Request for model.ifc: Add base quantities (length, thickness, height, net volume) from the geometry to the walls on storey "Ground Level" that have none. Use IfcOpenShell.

First a look at what the model holds.

```python
import ifcopenshell
import ifcopenshell.util.element
import ifcopenshell.util.unit

model = ifcopenshell.open("model.ifc")
print(model.schema)
for unit_type in ("LENGTHUNIT", "AREAUNIT", "VOLUMEUNIT"):
    print(unit_type, ifcopenshell.util.unit.calculate_unit_scale(model, unit_type))
storey = next(s for s in model.by_type("IfcBuildingStorey") if s.Name == "Ground Level")
walls = [e for e in ifcopenshell.util.element.get_decomposition(storey) if e.is_a("IfcWall")]
for e in sorted(walls, key=lambda e: e.id()):
    print(e.id(), e.is_a(), e.Name, list(ifcopenshell.util.element.get_psets(e, qtos_only=True)), sep=" | ")
```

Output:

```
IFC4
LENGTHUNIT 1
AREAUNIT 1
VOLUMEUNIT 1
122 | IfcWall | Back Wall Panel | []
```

```python
import ifcopenshell
import ifcopenshell.api.pset
import ifcopenshell.geom
import ifcopenshell.util.element
import ifcopenshell.util.shape
import ifcopenshell.util.unit

model = ifcopenshell.open("model.ifc")
unit_scale = ifcopenshell.util.unit.calculate_unit_scale(model)
volume_scale = ifcopenshell.util.unit.calculate_unit_scale(model, "VOLUMEUNIT")
settings = ifcopenshell.geom.settings()

storey = next(s for s in model.by_type("IfcBuildingStorey") if s.Name == "Ground Level")
walls = [e for e in ifcopenshell.util.element.get_decomposition(storey) if e.is_a("IfcWall")]

for e in sorted(walls, key=lambda e: e.id()):
    if ifcopenshell.util.element.get_psets(e, qtos_only=True, should_inherit=False):
        continue
    # Geometry comes back in metres, in the element's own axes.
    shape = ifcopenshell.geom.create_shape(settings, e)
    values = {
        "Length": ifcopenshell.util.shape.get_x(shape.geometry) / unit_scale,
        "Width": ifcopenshell.util.shape.get_y(shape.geometry) / unit_scale,
        "Height": ifcopenshell.util.shape.get_z(shape.geometry) / unit_scale,
        "NetVolume": ifcopenshell.util.shape.get_volume(shape.geometry) / volume_scale,
    }
    qto = ifcopenshell.api.pset.add_qto(model, product=e, name="Qto_WallBaseQuantities")
    ifcopenshell.api.pset.edit_qto(model, qto=qto, properties=values)
    print(e.id(), {k: round(v, 3) for k, v in values.items()})

model.write("model-out.ifc")
```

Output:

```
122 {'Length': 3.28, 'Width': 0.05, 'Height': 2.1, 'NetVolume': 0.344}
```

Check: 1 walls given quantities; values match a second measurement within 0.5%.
